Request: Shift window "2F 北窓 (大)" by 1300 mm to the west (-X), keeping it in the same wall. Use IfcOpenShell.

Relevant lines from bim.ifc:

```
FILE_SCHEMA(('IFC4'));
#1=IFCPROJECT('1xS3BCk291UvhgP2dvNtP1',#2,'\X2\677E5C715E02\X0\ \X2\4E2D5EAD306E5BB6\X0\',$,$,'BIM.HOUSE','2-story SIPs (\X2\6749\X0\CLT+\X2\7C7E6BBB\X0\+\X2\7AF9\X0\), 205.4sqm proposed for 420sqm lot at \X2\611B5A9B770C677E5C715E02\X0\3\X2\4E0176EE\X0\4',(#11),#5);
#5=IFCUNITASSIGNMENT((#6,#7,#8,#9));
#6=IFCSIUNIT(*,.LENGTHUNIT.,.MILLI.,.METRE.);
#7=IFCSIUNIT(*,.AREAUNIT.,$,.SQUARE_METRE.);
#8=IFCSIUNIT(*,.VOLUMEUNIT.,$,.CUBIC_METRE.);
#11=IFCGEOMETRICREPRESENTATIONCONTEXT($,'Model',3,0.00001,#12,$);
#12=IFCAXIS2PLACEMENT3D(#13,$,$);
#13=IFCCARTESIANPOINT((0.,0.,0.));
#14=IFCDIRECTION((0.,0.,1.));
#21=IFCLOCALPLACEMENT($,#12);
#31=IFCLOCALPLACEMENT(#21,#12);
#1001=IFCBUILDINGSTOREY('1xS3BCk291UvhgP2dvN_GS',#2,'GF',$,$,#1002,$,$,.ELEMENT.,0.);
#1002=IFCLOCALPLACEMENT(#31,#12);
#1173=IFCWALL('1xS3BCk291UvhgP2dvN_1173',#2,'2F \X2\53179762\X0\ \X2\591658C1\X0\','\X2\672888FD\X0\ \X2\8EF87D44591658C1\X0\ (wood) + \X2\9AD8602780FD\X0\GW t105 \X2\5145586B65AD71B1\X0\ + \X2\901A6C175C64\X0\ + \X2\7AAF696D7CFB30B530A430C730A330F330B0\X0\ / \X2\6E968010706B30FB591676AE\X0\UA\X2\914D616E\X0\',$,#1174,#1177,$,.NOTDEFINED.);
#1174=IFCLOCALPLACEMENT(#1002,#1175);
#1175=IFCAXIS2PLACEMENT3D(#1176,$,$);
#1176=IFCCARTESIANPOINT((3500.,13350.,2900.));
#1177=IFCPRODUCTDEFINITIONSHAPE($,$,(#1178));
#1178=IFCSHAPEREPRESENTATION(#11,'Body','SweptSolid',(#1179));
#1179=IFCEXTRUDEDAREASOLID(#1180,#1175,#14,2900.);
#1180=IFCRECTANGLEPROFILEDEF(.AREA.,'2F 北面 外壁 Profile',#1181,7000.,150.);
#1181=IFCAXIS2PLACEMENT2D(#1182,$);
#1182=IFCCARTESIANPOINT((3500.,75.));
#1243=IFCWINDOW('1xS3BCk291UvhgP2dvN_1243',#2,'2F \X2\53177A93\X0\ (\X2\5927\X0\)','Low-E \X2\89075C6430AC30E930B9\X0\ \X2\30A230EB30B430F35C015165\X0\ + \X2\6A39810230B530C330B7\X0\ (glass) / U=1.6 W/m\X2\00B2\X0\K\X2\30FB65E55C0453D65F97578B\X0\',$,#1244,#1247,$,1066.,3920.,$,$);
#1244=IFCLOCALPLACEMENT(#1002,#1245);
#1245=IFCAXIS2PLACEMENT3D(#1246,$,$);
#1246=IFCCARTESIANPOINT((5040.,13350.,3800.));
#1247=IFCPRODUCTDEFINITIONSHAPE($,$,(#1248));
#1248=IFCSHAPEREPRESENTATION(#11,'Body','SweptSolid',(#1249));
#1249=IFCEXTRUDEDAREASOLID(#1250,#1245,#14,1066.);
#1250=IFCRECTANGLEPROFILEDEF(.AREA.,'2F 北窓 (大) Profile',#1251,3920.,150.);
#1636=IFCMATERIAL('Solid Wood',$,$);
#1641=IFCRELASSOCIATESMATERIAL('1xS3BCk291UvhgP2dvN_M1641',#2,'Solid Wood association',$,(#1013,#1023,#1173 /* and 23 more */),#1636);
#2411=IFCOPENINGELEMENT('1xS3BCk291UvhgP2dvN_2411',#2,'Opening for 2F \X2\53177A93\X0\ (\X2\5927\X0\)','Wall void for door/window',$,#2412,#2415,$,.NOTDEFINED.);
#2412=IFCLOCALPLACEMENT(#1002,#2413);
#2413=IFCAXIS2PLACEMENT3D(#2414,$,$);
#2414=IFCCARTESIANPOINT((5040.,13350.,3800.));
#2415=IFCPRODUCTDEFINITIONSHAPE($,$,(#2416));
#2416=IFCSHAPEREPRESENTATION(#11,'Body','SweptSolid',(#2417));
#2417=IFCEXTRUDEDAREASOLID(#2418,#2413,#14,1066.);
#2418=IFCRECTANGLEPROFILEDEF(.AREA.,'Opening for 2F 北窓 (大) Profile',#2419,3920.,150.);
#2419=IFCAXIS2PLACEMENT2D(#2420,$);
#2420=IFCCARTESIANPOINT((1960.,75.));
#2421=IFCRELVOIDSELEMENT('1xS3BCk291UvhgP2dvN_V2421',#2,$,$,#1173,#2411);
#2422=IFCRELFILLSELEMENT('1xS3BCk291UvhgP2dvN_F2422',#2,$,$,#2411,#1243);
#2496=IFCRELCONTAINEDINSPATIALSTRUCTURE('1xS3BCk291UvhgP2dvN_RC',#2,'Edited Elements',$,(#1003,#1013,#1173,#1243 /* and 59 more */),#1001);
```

```python
import ifcopenshell
import ifcopenshell.api.geometry
import ifcopenshell.util.placement

model = ifcopenshell.open("bim.ifc")

window = model.by_guid("1xS3BCk291UvhgP2dvN_1243")
opening = window.FillsVoids[0].RelatingOpeningElement
wall = opening.VoidsElements[0].RelatingBuildingElement

wall_matrix = ifcopenshell.util.placement.get_local_placement(wall.ObjectPlacement)
shift = wall_matrix[:3, 0] * -1300.0
before = ifcopenshell.util.placement.get_local_placement(window.ObjectPlacement)[:3, 3].copy()

# The window is not placed relative to its opening, so move both.
for product in (opening, window):
    matrix = ifcopenshell.util.placement.get_local_placement(product.ObjectPlacement)
    matrix[:3, 3] += shift
    ifcopenshell.api.geometry.edit_object_placement(model, product=product, matrix=matrix, is_si=False)

after = ifcopenshell.util.placement.get_local_placement(window.ObjectPlacement)[:3, 3]
print("window moved by", (after - before).round(3) + 0.0)

model.write("bim_rev.ifc")
```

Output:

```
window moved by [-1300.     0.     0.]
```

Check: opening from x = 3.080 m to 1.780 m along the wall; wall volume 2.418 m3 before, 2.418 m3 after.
